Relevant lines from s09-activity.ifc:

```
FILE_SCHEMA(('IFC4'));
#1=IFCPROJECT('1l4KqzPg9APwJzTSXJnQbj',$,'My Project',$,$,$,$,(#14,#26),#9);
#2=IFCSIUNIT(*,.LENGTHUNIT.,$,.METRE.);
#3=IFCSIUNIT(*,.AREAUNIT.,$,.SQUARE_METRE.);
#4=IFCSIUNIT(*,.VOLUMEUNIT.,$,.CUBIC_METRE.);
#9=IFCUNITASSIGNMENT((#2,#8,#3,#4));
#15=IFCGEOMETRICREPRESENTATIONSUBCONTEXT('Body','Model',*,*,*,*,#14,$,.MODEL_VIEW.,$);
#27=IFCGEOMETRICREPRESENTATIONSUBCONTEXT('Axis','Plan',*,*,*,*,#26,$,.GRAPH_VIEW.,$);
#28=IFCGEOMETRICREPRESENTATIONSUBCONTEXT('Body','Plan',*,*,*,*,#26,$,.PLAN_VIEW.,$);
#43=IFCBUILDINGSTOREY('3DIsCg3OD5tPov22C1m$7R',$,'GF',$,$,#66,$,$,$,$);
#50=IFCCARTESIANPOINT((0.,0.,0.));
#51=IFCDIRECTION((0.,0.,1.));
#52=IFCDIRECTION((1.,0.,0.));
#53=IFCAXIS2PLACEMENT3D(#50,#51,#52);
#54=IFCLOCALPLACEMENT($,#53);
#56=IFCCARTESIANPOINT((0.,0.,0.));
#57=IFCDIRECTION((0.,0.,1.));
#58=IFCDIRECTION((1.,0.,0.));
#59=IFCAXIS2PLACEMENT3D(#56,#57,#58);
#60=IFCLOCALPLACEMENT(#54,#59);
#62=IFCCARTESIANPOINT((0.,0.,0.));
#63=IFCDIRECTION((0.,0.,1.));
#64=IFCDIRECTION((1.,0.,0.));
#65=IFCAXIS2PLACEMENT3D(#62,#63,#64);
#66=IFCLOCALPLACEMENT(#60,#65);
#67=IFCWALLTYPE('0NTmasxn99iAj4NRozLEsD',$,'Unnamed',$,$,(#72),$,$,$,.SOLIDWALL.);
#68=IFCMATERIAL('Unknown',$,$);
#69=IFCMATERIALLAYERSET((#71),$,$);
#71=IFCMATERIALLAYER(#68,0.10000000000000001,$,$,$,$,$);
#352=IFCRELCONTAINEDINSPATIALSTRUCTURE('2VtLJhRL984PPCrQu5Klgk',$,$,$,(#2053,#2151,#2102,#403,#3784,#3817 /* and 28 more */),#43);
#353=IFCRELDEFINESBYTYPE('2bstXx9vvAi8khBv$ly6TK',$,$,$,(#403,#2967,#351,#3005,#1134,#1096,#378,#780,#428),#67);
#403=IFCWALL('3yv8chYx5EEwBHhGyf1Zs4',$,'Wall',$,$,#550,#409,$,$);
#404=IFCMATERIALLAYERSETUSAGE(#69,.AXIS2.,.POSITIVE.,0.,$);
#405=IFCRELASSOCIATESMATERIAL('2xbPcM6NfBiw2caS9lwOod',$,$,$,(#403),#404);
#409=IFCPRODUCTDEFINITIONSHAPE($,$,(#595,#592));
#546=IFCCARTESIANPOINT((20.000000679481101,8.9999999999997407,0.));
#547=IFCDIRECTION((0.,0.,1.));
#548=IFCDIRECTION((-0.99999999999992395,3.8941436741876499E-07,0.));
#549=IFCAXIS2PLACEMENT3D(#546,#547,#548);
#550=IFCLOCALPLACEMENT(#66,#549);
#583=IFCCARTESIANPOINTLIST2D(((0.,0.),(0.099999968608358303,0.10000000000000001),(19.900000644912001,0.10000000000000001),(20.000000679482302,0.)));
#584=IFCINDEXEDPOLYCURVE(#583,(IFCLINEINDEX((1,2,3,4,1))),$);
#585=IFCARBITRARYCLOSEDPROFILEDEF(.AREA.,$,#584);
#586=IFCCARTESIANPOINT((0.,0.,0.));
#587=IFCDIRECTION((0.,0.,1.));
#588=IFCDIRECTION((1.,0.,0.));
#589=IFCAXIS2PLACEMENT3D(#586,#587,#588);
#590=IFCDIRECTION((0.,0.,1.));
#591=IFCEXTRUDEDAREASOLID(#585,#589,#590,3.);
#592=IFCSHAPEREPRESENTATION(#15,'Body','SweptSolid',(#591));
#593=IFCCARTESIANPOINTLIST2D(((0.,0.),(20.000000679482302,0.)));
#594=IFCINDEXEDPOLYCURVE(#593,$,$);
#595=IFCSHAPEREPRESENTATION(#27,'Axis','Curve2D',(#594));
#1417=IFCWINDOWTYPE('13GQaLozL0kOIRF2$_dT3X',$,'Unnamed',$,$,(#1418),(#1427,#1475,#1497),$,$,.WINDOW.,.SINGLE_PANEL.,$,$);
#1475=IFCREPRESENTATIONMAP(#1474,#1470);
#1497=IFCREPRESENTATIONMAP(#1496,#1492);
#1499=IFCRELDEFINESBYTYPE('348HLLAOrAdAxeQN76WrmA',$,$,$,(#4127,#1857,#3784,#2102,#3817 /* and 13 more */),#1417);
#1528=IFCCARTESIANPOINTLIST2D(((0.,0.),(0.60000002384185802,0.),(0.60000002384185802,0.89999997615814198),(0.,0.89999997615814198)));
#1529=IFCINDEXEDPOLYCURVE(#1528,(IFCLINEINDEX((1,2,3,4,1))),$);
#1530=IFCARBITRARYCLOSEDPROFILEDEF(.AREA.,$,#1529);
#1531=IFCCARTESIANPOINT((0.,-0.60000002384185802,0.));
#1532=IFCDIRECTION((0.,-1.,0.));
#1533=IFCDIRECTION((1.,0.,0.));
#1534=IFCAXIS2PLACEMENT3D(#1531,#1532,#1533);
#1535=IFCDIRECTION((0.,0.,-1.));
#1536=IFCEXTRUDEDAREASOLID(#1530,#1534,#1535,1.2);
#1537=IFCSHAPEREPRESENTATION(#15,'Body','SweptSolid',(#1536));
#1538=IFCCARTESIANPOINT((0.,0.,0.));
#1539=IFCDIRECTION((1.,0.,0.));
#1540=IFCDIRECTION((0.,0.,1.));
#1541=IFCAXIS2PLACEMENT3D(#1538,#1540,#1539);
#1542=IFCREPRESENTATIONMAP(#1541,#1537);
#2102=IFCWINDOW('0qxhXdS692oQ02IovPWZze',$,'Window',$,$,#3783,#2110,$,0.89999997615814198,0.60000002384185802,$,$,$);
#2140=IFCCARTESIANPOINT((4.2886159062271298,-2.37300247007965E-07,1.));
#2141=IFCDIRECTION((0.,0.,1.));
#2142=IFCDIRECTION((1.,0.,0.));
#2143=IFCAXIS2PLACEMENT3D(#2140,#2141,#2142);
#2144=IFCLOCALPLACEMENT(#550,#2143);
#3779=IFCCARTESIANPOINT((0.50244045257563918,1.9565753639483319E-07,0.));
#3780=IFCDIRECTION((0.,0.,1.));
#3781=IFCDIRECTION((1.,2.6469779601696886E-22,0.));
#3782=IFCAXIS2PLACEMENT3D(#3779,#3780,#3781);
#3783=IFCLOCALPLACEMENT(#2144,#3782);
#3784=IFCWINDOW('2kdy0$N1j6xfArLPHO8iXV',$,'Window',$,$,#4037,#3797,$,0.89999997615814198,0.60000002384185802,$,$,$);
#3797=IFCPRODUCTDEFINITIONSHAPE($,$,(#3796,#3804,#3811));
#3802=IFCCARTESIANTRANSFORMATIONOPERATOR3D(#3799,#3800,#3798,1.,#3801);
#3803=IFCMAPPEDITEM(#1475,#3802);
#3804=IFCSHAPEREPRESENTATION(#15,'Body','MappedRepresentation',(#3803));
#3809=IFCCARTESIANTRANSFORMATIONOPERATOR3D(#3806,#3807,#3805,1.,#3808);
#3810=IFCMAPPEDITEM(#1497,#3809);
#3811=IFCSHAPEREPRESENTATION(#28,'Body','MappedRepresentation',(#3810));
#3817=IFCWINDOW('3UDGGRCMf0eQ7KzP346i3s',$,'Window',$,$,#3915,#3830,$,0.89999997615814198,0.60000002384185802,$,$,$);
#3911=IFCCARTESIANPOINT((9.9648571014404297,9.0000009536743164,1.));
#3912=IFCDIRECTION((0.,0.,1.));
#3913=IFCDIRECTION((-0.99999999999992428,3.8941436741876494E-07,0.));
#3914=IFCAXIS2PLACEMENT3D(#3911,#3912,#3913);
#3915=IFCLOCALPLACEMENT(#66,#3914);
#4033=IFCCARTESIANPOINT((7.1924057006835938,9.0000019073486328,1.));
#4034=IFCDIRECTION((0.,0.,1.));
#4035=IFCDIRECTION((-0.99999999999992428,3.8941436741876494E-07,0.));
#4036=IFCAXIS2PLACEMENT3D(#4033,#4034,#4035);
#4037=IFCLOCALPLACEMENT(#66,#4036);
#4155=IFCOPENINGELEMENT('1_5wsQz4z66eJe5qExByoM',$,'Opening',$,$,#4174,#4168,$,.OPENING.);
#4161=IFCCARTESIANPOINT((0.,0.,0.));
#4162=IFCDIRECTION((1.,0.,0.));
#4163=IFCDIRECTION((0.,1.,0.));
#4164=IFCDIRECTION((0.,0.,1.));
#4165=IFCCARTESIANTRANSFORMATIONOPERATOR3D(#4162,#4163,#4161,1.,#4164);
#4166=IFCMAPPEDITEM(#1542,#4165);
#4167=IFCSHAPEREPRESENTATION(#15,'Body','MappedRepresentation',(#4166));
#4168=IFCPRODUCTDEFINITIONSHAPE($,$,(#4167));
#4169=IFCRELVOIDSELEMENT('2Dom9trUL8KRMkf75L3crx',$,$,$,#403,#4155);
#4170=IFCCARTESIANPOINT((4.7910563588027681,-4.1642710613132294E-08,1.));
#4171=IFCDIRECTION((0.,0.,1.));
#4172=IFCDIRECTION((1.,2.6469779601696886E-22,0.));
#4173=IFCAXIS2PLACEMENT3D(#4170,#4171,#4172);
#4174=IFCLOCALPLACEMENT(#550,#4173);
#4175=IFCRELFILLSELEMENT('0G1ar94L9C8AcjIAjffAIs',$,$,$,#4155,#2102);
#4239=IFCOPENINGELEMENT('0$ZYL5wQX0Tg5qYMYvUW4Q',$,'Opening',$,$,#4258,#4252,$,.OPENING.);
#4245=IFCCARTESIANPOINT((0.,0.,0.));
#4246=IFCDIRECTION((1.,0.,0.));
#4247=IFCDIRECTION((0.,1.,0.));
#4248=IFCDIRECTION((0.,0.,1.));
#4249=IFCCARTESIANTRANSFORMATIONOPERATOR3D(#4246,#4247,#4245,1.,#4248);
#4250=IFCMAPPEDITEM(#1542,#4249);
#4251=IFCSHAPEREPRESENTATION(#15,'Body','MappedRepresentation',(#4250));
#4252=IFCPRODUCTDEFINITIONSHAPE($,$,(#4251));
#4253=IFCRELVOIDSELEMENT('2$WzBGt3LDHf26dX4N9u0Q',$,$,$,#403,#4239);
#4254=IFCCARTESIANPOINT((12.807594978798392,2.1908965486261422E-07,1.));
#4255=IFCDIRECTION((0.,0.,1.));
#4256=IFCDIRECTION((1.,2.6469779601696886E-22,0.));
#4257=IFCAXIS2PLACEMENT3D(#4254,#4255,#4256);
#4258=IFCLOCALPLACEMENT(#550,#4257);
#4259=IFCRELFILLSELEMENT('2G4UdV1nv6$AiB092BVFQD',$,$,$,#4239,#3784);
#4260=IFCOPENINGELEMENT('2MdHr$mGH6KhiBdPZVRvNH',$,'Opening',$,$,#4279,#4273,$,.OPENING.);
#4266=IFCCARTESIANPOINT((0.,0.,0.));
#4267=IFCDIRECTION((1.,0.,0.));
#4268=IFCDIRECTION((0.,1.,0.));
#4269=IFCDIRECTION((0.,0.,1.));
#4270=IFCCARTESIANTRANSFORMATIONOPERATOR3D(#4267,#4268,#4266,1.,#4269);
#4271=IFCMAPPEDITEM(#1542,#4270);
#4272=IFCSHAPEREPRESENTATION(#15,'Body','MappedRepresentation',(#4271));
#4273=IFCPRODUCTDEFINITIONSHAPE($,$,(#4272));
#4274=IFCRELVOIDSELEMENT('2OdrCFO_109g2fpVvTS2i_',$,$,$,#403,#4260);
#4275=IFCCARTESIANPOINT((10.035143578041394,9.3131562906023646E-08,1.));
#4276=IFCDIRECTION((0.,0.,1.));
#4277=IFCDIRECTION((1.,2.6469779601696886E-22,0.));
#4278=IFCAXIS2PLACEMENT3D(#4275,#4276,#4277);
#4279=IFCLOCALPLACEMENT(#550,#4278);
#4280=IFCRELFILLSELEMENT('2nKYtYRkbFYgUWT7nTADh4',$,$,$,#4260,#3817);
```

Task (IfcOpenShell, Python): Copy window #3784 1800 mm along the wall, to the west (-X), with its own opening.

```python
import ifcopenshell
import ifcopenshell.api.feature
import ifcopenshell.api.geometry
import ifcopenshell.api.root
import ifcopenshell.geom
import ifcopenshell.util.element
import ifcopenshell.util.placement
import ifcopenshell.util.shape
import ifcopenshell.util.unit

model = ifcopenshell.open("s09-activity.ifc")
unit_scale = ifcopenshell.util.unit.calculate_unit_scale(model)
settings = ifcopenshell.geom.settings()


def volume(element):
    """Net volume in cubic metres, openings subtracted."""
    shape = ifcopenshell.geom.create_shape(settings, element)
    return ifcopenshell.util.shape.get_volume(shape.geometry)


window = model.by_guid("2kdy0$N1j6xfArLPHO8iXV")
opening = window.FillsVoids[0].RelatingOpeningElement
wall = opening.VoidsElements[0].RelatingBuildingElement
before = volume(wall)
shift = ifcopenshell.util.placement.get_local_placement(wall.ObjectPlacement)[:3, 0] * 1.8 / unit_scale

# copy_class copies the void relationship, type, container and properties, but no geometry.
new_opening = ifcopenshell.api.root.copy_class(model, product=opening)
new_opening.Representation = ifcopenshell.util.element.copy_deep(
    model, opening.Representation, exclude=["IfcGeometricRepresentationContext", "IfcRepresentationMap"]
)
new_window = ifcopenshell.api.root.copy_class(model, product=window)
new_window.Representation = ifcopenshell.util.element.copy_deep(
    model, window.Representation, exclude=["IfcGeometricRepresentationContext", "IfcRepresentationMap"]
)
ifcopenshell.api.feature.add_filling(model, opening=new_opening, element=new_window)

for old, new in ((opening, new_opening), (window, new_window)):
    matrix = ifcopenshell.util.placement.get_local_placement(old.ObjectPlacement)
    matrix[:3, 3] += shift
    ifcopenshell.api.geometry.edit_object_placement(model, product=new, matrix=matrix, is_si=False)

after = volume(wall)

print(f"wall volume {before:.3f} -> {after:.3f} m3")

model.write("s09-activity_rev.ifc")
```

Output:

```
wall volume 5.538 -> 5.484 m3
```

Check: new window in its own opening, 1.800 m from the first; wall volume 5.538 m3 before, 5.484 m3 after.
